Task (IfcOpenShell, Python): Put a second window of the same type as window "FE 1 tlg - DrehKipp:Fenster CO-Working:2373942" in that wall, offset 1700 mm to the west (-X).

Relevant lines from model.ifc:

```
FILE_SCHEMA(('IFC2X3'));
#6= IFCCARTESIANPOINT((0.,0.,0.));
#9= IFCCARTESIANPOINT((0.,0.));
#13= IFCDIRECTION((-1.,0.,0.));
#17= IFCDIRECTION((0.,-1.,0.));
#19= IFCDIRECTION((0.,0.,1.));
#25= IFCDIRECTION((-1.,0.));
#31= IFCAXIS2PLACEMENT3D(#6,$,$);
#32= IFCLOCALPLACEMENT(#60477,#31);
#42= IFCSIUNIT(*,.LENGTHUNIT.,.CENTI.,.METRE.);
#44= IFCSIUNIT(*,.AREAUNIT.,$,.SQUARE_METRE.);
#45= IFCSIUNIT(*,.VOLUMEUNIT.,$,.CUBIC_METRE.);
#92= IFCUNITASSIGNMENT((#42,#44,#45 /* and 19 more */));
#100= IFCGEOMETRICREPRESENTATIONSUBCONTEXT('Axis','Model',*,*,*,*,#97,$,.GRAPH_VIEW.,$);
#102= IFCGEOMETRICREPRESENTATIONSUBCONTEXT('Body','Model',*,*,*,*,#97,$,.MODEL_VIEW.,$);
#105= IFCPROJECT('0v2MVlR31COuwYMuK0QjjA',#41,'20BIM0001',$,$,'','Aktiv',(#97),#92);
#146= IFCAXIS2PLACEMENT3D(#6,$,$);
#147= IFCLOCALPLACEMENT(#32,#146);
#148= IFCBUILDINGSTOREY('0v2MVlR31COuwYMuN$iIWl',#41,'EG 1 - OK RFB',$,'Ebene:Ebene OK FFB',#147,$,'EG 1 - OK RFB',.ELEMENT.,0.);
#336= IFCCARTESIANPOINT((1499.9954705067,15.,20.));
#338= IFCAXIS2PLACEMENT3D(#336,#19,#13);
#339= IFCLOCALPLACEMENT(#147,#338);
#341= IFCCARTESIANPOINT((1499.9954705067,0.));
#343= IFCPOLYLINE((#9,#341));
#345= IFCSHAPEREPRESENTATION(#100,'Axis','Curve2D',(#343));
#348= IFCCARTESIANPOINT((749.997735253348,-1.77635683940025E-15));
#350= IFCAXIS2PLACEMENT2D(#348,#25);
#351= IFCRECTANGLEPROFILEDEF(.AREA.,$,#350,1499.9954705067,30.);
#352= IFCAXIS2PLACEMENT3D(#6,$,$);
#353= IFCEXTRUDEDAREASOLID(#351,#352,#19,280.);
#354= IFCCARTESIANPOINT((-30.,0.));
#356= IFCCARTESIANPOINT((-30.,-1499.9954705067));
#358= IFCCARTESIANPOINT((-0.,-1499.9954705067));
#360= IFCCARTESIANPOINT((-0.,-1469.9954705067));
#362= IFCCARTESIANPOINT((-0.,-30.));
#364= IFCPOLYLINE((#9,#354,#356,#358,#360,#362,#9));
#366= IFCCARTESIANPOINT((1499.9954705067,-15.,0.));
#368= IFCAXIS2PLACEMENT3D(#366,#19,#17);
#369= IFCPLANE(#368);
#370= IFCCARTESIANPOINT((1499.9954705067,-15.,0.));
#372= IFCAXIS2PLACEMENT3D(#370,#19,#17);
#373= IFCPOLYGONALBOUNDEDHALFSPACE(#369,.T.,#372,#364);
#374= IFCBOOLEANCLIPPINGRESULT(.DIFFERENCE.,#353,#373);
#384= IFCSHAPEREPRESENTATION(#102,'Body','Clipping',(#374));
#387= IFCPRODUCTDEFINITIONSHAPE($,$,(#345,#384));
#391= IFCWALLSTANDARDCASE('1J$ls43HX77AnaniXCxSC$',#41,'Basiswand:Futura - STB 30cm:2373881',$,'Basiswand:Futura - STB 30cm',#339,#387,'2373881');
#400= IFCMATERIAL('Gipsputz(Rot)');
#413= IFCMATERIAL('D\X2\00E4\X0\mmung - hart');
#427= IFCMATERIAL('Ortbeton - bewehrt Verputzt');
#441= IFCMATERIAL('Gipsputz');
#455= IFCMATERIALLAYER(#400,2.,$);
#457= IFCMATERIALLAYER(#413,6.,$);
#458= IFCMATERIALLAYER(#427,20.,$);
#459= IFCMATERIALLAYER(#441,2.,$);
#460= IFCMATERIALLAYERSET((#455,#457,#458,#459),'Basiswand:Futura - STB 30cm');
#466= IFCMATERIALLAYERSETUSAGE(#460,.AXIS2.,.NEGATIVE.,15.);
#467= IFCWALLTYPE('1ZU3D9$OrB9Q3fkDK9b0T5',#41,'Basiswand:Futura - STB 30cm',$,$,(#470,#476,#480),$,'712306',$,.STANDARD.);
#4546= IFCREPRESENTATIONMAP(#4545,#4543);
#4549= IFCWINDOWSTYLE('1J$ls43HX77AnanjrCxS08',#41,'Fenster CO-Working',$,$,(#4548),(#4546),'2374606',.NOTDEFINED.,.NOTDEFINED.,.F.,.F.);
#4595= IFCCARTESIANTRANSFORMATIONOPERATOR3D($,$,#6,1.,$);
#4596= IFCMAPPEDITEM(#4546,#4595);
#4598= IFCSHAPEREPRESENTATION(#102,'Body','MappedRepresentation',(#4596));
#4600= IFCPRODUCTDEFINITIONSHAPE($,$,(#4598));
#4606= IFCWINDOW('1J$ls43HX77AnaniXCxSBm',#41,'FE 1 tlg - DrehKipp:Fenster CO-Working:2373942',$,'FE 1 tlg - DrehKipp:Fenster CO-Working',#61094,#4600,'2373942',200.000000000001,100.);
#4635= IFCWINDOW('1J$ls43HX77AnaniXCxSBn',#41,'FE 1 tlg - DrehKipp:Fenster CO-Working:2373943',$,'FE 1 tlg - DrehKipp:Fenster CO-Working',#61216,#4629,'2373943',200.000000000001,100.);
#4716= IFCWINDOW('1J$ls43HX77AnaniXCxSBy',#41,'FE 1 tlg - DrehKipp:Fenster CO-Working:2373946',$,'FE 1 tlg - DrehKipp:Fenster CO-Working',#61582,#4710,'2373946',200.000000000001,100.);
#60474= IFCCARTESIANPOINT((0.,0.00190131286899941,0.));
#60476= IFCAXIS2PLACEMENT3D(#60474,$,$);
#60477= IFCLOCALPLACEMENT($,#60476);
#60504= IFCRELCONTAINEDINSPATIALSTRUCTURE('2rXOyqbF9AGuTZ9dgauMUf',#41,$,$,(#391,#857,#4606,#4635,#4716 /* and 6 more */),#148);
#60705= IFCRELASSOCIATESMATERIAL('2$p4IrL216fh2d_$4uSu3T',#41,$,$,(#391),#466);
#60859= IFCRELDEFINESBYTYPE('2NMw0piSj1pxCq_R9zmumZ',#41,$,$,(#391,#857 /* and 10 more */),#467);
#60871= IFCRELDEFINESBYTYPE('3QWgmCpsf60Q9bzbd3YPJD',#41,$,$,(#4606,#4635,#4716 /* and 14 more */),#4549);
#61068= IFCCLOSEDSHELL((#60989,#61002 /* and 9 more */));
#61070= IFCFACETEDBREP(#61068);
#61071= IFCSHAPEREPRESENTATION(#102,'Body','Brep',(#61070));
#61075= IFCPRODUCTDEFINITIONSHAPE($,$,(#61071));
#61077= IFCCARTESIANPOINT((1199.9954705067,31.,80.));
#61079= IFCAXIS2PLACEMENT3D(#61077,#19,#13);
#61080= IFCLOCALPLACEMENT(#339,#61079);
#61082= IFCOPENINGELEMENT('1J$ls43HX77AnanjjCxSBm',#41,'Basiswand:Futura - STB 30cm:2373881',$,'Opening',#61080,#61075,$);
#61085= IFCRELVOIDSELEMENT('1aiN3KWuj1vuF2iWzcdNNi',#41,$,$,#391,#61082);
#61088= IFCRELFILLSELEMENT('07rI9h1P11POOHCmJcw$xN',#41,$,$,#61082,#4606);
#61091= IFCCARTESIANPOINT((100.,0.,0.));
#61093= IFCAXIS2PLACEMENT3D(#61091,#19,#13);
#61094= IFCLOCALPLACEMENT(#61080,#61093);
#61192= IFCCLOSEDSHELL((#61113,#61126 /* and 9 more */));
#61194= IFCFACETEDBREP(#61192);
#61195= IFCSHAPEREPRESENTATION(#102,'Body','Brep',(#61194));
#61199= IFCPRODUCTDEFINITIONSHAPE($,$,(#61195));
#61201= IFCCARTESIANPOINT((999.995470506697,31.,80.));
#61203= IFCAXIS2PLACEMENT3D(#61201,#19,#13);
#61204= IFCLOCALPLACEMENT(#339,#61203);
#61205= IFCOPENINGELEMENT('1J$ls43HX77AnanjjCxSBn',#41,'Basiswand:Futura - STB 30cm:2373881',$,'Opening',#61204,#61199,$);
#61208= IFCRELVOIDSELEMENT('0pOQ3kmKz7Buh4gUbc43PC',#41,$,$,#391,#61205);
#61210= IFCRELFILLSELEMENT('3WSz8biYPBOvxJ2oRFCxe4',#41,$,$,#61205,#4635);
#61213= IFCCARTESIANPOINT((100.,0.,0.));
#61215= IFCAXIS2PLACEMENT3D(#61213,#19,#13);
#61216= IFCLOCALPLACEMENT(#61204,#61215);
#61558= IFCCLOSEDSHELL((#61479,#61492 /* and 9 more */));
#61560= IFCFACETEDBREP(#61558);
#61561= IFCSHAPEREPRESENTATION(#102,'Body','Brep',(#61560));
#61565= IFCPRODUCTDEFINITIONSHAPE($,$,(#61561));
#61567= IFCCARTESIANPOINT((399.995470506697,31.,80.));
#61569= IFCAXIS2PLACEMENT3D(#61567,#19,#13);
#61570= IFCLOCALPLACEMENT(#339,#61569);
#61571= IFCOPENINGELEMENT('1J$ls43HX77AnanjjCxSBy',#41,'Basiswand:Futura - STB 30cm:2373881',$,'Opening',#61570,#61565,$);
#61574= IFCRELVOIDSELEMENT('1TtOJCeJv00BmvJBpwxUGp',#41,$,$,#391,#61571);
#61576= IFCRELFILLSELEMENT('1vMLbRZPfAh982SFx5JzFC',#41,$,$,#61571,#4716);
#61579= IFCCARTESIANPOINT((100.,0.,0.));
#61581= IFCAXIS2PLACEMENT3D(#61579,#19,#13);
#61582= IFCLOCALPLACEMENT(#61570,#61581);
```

```python
import ifcopenshell
import ifcopenshell.api.feature
import ifcopenshell.api.geometry
import ifcopenshell.api.root
import ifcopenshell.geom
import ifcopenshell.util.element
import ifcopenshell.util.placement
import ifcopenshell.util.shape
import ifcopenshell.util.unit

model = ifcopenshell.open("model.ifc")
unit_scale = ifcopenshell.util.unit.calculate_unit_scale(model)
settings = ifcopenshell.geom.settings()


def volume(element):
    """Net volume in cubic metres, openings subtracted."""
    shape = ifcopenshell.geom.create_shape(settings, element)
    return ifcopenshell.util.shape.get_volume(shape.geometry)


def reuse_history(source, copy):
    """copy_class also copies each property set's owner history, people and application; keep the originals."""
    for rel in copy.IsDefinedBy:
        if rel.is_a("IfcRelDefinesByProperties") and (history := rel.RelatingPropertyDefinition.OwnerHistory):
            rel.RelatingPropertyDefinition.OwnerHistory = source.OwnerHistory
            ifcopenshell.util.element.remove_deep2(model, history)


window = model.by_id(4606)
opening = window.FillsVoids[0].RelatingOpeningElement
wall = opening.VoidsElements[0].RelatingBuildingElement
before = volume(wall)
shift = ifcopenshell.util.placement.get_local_placement(wall.ObjectPlacement)[:3, 0] * 1.7 / unit_scale

# copy_class copies the void relationship, type, container and properties, but no geometry.
new_opening = ifcopenshell.api.root.copy_class(model, product=opening)
new_opening.Representation = ifcopenshell.util.element.copy_deep(
    model, opening.Representation, exclude=["IfcGeometricRepresentationContext", "IfcRepresentationMap"]
)
new_opening.Name = "Basiswand:Futura - STB 30cm"
new_window = ifcopenshell.api.root.copy_class(model, product=window)
new_window.Representation = ifcopenshell.util.element.copy_deep(
    model, window.Representation, exclude=["IfcGeometricRepresentationContext", "IfcRepresentationMap"]
)
new_window.Name = "FE 1 tlg - DrehKipp:Fenster CO-Working"
new_window.Tag = None
reuse_history(window, new_window)
fills = ifcopenshell.api.feature.add_filling(model, opening=new_opening, element=new_window)
fills.OwnerHistory = new_window.OwnerHistory  # required in IFC2X3

for old, new in ((opening, new_opening), (window, new_window)):
    matrix = ifcopenshell.util.placement.get_local_placement(old.ObjectPlacement)
    matrix[:3, 3] += shift
    ifcopenshell.api.geometry.edit_object_placement(model, product=new, matrix=matrix, is_si=False)

after = volume(wall)

print(f"wall volume {before:.3f} -> {after:.3f} m3")

model.write("model_rev.ifc")
```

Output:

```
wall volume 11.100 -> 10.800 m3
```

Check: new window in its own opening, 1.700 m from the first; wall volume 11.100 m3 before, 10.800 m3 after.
